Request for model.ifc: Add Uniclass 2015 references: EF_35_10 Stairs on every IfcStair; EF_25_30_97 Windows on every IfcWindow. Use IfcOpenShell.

First a look at what the model holds.

```python
import ifcopenshell

model = ifcopenshell.open("model.ifc")
print(model.schema)
print("classifications:", [c.Name for c in model.by_type("IfcClassification")])
for ifc_class in ("IfcDoor", "IfcRoof", "IfcStair", "IfcWall", "IfcWindow"):
    print(ifc_class, len(model.by_type(ifc_class)))
```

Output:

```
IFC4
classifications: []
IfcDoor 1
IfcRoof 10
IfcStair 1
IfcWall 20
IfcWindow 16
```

```python
import ifcopenshell
import ifcopenshell.api.classification

model = ifcopenshell.open("model.ifc")

system = ifcopenshell.api.classification.add_classification(model, classification="Uniclass 2015")

codes = {
    "IfcStair": ("EF_35_10", "Stairs"),
    "IfcWindow": ("EF_25_30_97", "Windows"),
}
for ifc_class, (code, name) in codes.items():
    products = model.by_type(ifc_class)
    ifcopenshell.api.classification.add_reference(
        model, products=products, classification=system, identification=code, name=name
    )
    print(code, len(products))

model.write("model_v2.ifc")
```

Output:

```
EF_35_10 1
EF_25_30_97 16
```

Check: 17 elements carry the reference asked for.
